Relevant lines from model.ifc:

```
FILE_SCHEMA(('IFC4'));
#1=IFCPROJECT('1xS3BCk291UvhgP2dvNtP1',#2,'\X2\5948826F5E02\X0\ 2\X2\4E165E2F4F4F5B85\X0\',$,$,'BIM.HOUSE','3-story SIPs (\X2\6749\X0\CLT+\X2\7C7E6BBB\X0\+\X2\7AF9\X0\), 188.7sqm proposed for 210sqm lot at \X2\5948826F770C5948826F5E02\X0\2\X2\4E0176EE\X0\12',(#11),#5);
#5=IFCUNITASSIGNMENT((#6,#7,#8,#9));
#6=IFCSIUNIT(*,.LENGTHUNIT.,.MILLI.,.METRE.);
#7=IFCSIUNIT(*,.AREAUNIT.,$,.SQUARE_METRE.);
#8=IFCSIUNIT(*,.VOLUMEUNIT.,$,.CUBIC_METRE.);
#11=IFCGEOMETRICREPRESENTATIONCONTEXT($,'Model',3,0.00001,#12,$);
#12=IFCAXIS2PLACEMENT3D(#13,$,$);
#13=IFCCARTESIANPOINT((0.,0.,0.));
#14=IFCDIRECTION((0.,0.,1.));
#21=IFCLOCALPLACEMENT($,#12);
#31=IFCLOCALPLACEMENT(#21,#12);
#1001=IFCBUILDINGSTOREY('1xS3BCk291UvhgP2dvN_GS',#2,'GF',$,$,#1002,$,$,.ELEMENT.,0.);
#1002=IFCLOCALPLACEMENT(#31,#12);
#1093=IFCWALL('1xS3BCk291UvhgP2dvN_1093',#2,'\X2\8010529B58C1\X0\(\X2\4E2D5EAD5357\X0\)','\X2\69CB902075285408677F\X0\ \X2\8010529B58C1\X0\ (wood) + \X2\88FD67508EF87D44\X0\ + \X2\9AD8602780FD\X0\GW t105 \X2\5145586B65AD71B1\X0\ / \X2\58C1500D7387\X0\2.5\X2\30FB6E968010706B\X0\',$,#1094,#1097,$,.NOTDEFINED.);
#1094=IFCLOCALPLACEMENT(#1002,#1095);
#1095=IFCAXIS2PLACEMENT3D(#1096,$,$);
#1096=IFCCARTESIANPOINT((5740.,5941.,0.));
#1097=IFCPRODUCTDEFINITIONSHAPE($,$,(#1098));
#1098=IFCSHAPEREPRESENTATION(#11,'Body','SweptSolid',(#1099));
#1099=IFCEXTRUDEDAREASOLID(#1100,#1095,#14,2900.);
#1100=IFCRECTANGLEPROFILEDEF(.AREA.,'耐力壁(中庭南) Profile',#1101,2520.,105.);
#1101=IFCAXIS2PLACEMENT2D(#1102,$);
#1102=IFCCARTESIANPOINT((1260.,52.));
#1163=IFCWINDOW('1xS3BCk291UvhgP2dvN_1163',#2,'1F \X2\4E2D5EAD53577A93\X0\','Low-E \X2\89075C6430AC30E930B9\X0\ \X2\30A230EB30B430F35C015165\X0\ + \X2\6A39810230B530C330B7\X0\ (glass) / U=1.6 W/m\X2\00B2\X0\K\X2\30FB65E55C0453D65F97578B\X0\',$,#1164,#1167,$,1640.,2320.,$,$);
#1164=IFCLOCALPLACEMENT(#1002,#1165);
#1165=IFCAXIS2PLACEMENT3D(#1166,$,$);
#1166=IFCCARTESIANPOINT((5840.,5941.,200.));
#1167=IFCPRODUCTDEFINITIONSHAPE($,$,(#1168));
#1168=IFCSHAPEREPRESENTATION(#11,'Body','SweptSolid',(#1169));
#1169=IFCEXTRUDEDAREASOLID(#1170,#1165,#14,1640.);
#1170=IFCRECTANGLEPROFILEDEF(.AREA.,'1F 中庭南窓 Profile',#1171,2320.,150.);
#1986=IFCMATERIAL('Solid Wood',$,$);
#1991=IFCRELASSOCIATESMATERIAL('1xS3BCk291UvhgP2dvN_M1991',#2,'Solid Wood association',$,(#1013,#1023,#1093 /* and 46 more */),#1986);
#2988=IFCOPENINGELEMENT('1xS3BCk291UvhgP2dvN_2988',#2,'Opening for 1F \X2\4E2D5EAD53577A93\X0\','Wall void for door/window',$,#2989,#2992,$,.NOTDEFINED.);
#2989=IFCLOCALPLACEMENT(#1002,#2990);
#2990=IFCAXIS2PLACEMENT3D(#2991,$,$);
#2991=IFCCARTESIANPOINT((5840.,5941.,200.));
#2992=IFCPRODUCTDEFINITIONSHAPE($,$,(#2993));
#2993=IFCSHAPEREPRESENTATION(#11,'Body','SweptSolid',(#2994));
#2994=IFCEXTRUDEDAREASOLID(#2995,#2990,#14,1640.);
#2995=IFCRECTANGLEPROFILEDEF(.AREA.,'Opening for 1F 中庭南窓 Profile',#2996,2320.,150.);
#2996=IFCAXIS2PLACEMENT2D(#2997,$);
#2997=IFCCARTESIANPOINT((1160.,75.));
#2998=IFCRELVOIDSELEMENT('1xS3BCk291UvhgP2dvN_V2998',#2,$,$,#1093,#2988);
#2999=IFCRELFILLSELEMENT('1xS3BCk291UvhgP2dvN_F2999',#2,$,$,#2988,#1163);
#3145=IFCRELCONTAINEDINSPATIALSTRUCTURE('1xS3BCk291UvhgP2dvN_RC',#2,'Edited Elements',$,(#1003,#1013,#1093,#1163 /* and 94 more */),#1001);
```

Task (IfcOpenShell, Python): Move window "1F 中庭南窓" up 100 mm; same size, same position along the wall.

```python
import numpy as np
import ifcopenshell
import ifcopenshell.api.geometry
import ifcopenshell.util.placement
import ifcopenshell.util.unit

model = ifcopenshell.open("model.ifc")
unit_scale = ifcopenshell.util.unit.calculate_unit_scale(model)

window = model.by_guid("1xS3BCk291UvhgP2dvN_1163")
opening = window.FillsVoids[0].RelatingOpeningElement
dz = 100.0

shift = np.array([0.0, 0.0, dz])
# The window is not placed relative to its opening, so move both.
for product in (opening, window):
    matrix = ifcopenshell.util.placement.get_local_placement(product.ObjectPlacement)
    matrix[:3, 3] += shift
    ifcopenshell.api.geometry.edit_object_placement(model, product=product, matrix=matrix, is_si=False)

print(f"moved by {dz * unit_scale:+.3f} m")

model.write("model_updated.ifc")
```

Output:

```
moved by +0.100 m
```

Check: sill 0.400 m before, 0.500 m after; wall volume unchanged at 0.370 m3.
